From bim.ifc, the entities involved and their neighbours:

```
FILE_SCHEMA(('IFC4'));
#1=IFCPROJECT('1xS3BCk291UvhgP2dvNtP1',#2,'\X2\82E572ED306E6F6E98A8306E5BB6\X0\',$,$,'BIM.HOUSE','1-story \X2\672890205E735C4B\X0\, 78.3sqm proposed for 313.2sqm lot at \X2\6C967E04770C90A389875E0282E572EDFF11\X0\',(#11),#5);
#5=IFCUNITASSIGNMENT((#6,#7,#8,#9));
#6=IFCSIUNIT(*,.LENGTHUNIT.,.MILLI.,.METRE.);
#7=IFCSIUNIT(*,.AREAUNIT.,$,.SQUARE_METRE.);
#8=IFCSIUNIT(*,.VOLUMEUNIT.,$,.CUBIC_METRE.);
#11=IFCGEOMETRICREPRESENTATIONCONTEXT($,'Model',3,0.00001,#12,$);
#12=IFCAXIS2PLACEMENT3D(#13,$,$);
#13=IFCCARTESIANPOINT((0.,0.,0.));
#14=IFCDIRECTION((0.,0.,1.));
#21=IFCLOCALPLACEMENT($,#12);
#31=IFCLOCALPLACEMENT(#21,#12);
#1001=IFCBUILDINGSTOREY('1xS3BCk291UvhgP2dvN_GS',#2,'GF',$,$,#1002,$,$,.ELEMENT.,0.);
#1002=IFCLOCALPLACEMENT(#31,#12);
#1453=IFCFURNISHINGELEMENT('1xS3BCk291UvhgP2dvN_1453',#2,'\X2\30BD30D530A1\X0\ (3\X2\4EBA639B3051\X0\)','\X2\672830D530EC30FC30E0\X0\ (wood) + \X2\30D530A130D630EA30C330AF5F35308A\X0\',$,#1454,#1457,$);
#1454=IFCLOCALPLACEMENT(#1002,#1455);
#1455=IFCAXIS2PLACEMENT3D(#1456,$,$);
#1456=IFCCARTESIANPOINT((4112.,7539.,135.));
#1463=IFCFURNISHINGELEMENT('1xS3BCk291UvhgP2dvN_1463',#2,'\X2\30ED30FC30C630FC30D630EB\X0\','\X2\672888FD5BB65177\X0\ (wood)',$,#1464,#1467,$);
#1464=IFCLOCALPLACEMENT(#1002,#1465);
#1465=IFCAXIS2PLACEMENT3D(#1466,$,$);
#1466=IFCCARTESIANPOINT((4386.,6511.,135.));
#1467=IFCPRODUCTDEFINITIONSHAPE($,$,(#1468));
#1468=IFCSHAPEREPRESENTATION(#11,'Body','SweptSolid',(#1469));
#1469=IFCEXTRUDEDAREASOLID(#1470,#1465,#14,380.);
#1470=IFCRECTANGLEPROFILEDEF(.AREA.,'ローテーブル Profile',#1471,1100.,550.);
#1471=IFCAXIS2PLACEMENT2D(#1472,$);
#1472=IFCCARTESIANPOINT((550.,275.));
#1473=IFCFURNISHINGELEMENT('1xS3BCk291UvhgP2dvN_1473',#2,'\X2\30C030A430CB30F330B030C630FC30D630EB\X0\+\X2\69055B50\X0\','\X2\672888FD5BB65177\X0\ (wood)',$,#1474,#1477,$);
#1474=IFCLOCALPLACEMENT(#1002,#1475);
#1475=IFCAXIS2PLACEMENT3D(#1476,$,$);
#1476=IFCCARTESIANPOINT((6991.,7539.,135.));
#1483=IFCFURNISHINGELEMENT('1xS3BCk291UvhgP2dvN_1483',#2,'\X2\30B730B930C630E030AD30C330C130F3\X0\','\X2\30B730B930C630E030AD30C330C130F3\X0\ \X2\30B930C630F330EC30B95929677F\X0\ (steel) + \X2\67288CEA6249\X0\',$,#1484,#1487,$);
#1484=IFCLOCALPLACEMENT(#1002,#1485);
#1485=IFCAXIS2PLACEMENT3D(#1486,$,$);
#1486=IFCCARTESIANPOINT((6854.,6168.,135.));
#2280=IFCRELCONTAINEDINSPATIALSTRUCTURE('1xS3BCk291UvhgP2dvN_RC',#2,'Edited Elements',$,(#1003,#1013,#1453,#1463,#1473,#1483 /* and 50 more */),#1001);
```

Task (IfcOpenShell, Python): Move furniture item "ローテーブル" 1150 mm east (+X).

```python
import ifcopenshell
import ifcopenshell.api.geometry
import ifcopenshell.util.placement
import ifcopenshell.util.unit

model = ifcopenshell.open("bim.ifc")
unit_scale = ifcopenshell.util.unit.calculate_unit_scale(model)

item = model.by_guid("1xS3BCk291UvhgP2dvN_1463")
matrix = ifcopenshell.util.placement.get_local_placement(item.ObjectPlacement)
matrix[0, 3] += 1.15 / unit_scale
ifcopenshell.api.geometry.edit_object_placement(model, product=item, matrix=matrix, is_si=False)

print(ifcopenshell.util.placement.get_local_placement(item.ObjectPlacement).round(3) + 0.0)

model.write("bim_edited.ifc")
```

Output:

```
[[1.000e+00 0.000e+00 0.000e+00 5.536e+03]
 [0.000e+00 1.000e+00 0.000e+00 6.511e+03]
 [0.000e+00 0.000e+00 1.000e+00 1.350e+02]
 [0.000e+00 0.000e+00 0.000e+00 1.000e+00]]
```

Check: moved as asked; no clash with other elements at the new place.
